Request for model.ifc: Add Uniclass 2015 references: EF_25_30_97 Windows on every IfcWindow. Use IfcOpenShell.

First a look at what the model holds.

```python
import ifcopenshell

model = ifcopenshell.open("model.ifc")
print(model.schema)
print("classifications:", [c.Name for c in model.by_type("IfcClassification")])
for ifc_class in ("IfcDoor", "IfcRoof", "IfcStair", "IfcWall", "IfcWindow"):
    print(ifc_class, len(model.by_type(ifc_class)))
```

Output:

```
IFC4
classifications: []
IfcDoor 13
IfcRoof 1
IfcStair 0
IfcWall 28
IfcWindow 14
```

```python
import ifcopenshell
import ifcopenshell.api.classification

model = ifcopenshell.open("model.ifc")

system = ifcopenshell.api.classification.add_classification(model, classification="Uniclass 2015")

codes = {
    "IfcWindow": ("EF_25_30_97", "Windows"),
}
for ifc_class, (code, name) in codes.items():
    products = model.by_type(ifc_class)
    ifcopenshell.api.classification.add_reference(
        model, products=products, classification=system, identification=code, name=name
    )
    print(code, len(products))

model.write("model_rev.ifc")
```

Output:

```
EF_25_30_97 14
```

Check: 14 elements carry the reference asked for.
